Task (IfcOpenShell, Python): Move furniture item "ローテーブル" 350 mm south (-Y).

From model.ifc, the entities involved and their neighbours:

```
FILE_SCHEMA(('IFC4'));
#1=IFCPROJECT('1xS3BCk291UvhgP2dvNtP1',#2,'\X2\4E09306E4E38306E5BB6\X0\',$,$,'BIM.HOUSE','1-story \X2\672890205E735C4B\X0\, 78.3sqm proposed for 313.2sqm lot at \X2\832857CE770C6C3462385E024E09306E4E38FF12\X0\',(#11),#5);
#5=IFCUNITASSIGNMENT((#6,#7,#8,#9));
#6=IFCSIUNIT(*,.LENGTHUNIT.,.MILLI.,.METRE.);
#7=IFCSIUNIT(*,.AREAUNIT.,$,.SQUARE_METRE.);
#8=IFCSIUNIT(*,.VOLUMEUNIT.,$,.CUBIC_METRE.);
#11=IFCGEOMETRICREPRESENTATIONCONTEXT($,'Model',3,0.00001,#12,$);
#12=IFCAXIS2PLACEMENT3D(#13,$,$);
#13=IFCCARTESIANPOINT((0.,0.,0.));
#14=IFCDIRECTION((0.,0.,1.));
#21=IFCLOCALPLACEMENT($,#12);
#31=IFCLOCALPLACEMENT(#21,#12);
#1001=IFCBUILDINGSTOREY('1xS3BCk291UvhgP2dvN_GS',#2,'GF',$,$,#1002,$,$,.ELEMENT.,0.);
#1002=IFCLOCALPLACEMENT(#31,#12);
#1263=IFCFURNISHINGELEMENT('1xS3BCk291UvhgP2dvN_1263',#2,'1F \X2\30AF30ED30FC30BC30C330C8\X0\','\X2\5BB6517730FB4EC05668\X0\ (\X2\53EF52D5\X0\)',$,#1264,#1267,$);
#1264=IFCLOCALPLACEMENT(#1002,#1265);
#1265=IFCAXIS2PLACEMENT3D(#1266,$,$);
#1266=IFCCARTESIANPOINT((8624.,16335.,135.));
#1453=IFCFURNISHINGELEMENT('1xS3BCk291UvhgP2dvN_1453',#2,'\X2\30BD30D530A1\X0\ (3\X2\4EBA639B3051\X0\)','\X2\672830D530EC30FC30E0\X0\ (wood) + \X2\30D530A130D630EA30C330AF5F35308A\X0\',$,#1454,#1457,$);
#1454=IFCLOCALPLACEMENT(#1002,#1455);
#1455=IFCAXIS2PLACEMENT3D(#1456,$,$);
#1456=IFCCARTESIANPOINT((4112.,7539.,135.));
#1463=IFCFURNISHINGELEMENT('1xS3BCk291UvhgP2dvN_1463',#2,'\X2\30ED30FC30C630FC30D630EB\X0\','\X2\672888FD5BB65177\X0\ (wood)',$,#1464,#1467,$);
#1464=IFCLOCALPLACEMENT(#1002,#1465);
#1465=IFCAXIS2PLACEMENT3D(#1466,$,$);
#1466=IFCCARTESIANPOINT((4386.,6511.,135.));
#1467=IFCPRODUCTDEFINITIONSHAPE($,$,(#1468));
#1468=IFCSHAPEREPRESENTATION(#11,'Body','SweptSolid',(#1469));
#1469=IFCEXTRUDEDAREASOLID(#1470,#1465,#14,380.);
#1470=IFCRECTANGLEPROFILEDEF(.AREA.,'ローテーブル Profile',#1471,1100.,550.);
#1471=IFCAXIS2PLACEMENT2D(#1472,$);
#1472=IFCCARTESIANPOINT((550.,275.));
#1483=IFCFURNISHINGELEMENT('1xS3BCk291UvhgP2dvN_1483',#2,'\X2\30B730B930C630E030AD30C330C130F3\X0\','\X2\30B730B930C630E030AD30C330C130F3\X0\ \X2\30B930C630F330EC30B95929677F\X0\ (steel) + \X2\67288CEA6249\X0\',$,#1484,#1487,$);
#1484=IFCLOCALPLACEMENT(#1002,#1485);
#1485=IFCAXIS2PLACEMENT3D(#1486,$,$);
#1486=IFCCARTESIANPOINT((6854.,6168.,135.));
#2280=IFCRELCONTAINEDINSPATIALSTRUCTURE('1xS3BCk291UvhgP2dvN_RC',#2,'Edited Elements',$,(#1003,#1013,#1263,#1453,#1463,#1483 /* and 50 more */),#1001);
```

```python
import ifcopenshell
import ifcopenshell.api.geometry
import ifcopenshell.util.placement
import ifcopenshell.util.unit

model = ifcopenshell.open("model.ifc")
unit_scale = ifcopenshell.util.unit.calculate_unit_scale(model)

item = model.by_guid("1xS3BCk291UvhgP2dvN_1463")
matrix = ifcopenshell.util.placement.get_local_placement(item.ObjectPlacement)
matrix[1, 3] -= 0.35 / unit_scale
ifcopenshell.api.geometry.edit_object_placement(model, product=item, matrix=matrix, is_si=False)

print(ifcopenshell.util.placement.get_local_placement(item.ObjectPlacement).round(3) + 0.0)

model.write("model_v2.ifc")
```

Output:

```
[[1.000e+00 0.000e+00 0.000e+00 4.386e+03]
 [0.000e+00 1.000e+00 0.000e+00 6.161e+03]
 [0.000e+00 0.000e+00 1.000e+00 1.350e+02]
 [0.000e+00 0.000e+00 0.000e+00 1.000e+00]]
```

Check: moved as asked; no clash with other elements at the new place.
